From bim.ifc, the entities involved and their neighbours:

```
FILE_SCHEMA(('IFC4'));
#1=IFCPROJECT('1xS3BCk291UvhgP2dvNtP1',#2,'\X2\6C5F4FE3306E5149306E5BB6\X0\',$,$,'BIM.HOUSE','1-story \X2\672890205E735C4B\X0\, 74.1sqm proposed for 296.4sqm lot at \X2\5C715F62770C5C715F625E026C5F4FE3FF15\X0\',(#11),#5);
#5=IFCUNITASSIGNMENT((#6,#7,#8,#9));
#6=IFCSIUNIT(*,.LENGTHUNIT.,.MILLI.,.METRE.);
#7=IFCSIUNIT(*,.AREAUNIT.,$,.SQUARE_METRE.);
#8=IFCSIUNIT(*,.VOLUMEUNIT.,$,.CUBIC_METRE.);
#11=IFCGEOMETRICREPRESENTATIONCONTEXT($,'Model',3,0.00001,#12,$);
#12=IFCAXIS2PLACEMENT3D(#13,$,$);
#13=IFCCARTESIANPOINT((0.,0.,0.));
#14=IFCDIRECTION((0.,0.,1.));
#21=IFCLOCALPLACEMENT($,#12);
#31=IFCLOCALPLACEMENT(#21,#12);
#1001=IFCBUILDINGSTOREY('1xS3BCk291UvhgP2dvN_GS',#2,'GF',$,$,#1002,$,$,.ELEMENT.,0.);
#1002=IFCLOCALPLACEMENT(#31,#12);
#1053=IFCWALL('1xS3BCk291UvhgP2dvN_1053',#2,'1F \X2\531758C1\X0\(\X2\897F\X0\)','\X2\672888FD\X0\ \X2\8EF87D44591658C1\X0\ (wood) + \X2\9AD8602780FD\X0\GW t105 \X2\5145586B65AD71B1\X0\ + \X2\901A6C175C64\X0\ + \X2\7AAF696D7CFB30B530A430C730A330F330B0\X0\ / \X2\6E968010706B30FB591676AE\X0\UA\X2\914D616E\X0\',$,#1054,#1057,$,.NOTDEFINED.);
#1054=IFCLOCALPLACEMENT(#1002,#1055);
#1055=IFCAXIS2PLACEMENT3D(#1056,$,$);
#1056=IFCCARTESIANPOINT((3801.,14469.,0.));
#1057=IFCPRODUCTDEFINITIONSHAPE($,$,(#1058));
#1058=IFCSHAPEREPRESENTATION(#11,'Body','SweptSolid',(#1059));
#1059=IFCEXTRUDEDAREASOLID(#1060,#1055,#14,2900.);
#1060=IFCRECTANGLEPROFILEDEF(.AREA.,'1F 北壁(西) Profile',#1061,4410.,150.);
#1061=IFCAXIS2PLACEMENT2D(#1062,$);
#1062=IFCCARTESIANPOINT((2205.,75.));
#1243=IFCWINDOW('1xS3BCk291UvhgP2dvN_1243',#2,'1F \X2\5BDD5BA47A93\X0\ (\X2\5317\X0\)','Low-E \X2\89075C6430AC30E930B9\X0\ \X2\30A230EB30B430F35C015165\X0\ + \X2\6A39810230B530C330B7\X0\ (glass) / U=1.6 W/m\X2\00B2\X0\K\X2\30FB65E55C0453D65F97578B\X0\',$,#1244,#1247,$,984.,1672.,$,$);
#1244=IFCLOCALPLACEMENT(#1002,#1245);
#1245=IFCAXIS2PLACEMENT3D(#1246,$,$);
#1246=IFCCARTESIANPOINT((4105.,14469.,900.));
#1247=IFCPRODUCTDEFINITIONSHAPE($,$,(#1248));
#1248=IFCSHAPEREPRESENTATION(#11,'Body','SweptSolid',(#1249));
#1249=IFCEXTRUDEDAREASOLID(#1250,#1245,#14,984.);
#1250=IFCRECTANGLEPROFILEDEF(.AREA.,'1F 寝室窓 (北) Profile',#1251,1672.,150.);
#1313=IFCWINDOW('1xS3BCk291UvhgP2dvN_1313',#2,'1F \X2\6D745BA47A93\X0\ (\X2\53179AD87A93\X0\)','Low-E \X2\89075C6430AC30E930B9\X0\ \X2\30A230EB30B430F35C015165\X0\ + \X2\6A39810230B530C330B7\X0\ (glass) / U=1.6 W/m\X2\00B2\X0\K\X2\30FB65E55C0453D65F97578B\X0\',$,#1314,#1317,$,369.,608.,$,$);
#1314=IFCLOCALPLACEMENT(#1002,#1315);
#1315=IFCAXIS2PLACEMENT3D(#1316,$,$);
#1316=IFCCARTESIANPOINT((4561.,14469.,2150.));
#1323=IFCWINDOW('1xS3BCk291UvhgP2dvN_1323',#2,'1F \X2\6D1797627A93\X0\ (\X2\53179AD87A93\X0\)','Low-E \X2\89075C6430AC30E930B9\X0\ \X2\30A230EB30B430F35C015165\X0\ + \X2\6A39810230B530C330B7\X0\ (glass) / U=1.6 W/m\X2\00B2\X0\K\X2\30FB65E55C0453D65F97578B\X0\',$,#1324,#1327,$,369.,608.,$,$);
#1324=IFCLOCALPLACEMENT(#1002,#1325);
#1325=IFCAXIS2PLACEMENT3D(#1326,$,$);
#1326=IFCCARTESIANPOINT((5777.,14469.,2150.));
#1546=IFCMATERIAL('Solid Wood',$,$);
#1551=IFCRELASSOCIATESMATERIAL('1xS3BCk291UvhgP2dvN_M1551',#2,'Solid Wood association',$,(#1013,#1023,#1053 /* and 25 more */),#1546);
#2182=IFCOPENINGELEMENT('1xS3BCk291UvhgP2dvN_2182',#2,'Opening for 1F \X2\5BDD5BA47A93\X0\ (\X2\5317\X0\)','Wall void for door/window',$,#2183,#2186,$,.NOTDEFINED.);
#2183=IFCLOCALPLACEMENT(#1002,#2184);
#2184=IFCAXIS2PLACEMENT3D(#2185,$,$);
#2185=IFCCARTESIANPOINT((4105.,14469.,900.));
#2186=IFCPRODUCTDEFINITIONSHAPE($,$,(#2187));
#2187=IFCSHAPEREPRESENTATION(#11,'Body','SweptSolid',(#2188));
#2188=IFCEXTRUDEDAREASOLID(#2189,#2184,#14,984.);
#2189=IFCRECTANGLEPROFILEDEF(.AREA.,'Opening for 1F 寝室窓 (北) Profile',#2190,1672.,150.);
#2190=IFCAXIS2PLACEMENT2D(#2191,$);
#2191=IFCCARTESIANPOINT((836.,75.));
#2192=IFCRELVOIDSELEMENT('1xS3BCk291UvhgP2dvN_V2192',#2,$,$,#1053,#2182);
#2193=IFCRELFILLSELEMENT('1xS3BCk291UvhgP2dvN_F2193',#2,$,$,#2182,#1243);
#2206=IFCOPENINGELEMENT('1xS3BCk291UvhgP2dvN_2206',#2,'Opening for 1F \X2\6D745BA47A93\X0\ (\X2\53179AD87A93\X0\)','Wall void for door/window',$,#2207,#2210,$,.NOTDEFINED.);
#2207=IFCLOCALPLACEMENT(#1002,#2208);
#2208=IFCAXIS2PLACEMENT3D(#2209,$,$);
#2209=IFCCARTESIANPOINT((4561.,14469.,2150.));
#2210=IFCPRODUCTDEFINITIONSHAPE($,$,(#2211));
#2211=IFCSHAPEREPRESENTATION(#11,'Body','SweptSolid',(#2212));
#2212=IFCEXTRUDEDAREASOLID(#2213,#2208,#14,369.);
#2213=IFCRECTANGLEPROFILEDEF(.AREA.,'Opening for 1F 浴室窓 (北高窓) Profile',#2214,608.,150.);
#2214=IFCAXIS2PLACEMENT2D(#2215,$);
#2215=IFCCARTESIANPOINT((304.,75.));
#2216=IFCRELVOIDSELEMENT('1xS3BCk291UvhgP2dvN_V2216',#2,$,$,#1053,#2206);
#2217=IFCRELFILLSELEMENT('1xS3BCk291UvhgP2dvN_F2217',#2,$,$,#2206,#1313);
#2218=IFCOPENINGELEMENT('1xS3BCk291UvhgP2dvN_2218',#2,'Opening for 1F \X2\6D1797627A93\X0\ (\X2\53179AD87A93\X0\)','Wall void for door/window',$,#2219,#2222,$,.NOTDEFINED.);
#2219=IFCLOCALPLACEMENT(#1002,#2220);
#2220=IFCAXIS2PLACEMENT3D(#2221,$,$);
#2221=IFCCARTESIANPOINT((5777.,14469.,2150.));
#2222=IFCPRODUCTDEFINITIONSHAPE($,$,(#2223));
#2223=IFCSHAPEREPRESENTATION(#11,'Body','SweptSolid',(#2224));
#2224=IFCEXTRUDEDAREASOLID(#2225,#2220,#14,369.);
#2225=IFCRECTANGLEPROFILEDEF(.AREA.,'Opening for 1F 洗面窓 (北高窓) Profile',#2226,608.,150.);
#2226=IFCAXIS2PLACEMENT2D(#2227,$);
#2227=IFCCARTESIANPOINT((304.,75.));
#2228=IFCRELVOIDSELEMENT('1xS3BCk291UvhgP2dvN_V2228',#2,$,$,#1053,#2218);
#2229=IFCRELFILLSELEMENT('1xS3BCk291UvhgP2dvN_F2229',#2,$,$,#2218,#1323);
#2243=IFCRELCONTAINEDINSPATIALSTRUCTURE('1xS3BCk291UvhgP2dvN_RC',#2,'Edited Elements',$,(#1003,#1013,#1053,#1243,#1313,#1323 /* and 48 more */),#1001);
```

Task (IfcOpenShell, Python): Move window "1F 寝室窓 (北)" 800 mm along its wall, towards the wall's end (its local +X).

```python
import ifcopenshell
import ifcopenshell.api.geometry
import ifcopenshell.util.placement

model = ifcopenshell.open("bim.ifc")

window = model.by_id(1243)
opening = window.FillsVoids[0].RelatingOpeningElement
wall = opening.VoidsElements[0].RelatingBuildingElement

wall_matrix = ifcopenshell.util.placement.get_local_placement(wall.ObjectPlacement)
shift = wall_matrix[:3, 0] * 800.0
before = ifcopenshell.util.placement.get_local_placement(window.ObjectPlacement)[:3, 3].copy()

# The window is not placed relative to its opening, so move both.
for product in (opening, window):
    matrix = ifcopenshell.util.placement.get_local_placement(product.ObjectPlacement)
    matrix[:3, 3] += shift
    ifcopenshell.api.geometry.edit_object_placement(model, product=product, matrix=matrix, is_si=False)

after = ifcopenshell.util.placement.get_local_placement(window.ObjectPlacement)[:3, 3]
print("window moved by", (after - before).round(3) + 0.0)

model.write("bim-out.ifc")
```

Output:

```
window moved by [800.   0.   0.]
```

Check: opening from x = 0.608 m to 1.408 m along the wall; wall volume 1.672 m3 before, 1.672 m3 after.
